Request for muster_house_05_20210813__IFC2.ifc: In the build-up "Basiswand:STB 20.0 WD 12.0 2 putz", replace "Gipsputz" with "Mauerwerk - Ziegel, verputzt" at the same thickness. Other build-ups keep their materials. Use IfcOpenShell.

First a look at what the model holds.

```python
import ifcopenshell
import ifcopenshell.util.element

model = ifcopenshell.open("muster_house_05_20210813__IFC2.ifc")
print(model.schema)
for layer_set in model.by_type("IfcMaterialLayerSet"):
    if layer_set.LayerSetName == "Basiswand:STB 20.0 WD 12.0 2 putz":
        for layer in layer_set.MaterialLayers:
            print(layer.id(), layer.Material and layer.Material.Name, layer.LayerThickness, sep=" | ")
        print(len(ifcopenshell.util.element.get_elements_by_material(model, layer_set)), "elements and types use it")
print(sorted(m.Name for m in model.by_type("IfcMaterial") if m.Name)[:60])
```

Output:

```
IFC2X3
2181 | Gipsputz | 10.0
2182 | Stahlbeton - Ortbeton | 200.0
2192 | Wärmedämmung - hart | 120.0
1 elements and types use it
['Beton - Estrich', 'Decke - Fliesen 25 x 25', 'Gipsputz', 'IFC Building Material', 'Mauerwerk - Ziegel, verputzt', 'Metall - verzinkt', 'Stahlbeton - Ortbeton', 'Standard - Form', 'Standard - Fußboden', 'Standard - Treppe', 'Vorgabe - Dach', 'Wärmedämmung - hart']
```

```python
import ifcopenshell
import ifcopenshell.api.material

model = ifcopenshell.open("muster_house_05_20210813__IFC2.ifc")

layer_set = next(s for s in model.by_type("IfcMaterialLayerSet") if s.LayerSetName == "Basiswand:STB 20.0 WD 12.0 2 putz")
layer = next(l for l in layer_set.MaterialLayers if l.Material and l.Material.Name == "Gipsputz")
material = next(m for m in model.by_type("IfcMaterial") if m.Name == "Mauerwerk - Ziegel, verputzt")

# Point this one layer at the other material; renaming the old one would change it everywhere.
ifcopenshell.api.material.edit_layer(model, layer=layer, attributes={}, material=material)

print([l.Material.Name if l.Material else None for l in layer_set.MaterialLayers])

model.write("muster_house_05_20210813__IFC2_rev.ifc")
```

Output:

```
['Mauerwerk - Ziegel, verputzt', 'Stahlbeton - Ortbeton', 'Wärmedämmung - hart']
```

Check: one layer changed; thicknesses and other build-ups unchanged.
